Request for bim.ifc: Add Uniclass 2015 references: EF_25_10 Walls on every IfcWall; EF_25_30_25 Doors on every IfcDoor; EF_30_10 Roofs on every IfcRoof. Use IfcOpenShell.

First a look at what the model holds.

```python
import ifcopenshell

model = ifcopenshell.open("bim.ifc")
print(model.schema)
print("classifications:", [c.Name for c in model.by_type("IfcClassification")])
for ifc_class in ("IfcDoor", "IfcRoof", "IfcStair", "IfcWall", "IfcWindow"):
    print(ifc_class, len(model.by_type(ifc_class)))
```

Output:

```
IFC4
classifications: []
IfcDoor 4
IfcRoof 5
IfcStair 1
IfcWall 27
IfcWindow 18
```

```python
import ifcopenshell
import ifcopenshell.api.classification

model = ifcopenshell.open("bim.ifc")

system = ifcopenshell.api.classification.add_classification(model, classification="Uniclass 2015")

codes = {
    "IfcWall": ("EF_25_10", "Walls"),
    "IfcDoor": ("EF_25_30_25", "Doors"),
    "IfcRoof": ("EF_30_10", "Roofs"),
}
for ifc_class, (code, name) in codes.items():
    products = model.by_type(ifc_class)
    ifcopenshell.api.classification.add_reference(
        model, products=products, classification=system, identification=code, name=name
    )
    print(code, len(products))

model.write("bim_edited.ifc")
```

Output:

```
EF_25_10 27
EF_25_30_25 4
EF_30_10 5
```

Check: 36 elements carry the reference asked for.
